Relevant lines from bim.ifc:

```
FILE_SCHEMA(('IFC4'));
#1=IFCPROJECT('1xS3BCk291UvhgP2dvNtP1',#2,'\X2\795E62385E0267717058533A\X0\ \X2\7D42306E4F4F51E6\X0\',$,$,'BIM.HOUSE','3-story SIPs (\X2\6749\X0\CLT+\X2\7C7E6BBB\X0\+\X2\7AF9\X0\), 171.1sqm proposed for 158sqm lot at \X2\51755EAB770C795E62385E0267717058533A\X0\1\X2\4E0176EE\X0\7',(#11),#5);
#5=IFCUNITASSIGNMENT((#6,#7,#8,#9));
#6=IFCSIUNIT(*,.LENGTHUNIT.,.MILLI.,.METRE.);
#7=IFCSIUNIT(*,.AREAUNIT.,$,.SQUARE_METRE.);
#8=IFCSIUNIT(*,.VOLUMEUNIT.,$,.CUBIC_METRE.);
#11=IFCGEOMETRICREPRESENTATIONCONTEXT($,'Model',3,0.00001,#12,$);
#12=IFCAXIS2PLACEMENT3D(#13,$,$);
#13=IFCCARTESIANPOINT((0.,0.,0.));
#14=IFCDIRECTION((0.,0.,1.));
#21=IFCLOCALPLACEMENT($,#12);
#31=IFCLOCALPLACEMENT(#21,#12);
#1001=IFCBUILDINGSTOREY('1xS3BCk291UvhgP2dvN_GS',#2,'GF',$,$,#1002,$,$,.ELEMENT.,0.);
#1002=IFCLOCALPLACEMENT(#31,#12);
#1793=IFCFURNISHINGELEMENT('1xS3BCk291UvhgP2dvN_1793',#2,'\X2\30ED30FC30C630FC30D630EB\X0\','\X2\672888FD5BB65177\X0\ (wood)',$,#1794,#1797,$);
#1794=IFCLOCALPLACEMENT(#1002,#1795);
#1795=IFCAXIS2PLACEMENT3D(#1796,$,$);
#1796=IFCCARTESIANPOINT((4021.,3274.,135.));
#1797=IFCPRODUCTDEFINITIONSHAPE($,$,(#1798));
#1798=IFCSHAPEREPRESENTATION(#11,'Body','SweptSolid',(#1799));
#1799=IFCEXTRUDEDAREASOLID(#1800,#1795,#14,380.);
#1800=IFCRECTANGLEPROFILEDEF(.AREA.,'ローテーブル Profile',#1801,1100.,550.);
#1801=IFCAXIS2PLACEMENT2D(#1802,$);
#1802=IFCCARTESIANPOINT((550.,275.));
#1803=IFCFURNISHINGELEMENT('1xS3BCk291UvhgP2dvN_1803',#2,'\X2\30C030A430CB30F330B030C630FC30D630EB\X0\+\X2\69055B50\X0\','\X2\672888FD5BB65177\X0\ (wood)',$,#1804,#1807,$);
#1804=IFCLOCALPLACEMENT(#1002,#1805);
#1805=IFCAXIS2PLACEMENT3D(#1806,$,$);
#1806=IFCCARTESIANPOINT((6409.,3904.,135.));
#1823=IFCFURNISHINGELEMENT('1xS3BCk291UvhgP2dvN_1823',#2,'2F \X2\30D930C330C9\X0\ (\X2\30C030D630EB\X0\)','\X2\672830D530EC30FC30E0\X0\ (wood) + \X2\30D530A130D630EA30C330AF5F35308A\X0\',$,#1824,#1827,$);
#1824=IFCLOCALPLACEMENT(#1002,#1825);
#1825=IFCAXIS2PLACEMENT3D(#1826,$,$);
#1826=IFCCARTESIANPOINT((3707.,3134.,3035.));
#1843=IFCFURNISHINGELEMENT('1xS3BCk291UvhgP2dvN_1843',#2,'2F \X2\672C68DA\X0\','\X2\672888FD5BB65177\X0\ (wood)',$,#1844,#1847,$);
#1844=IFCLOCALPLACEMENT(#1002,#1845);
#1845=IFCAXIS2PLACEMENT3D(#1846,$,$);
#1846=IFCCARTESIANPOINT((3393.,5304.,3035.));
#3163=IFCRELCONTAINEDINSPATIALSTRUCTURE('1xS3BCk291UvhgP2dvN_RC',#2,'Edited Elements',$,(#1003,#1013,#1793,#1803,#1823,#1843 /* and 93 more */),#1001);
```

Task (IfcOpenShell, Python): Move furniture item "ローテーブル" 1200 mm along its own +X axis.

```python
import ifcopenshell
import ifcopenshell.api.geometry
import ifcopenshell.util.placement
import ifcopenshell.util.unit

model = ifcopenshell.open("bim.ifc")
unit_scale = ifcopenshell.util.unit.calculate_unit_scale(model)

item = model.by_id(1793)
matrix = ifcopenshell.util.placement.get_local_placement(item.ObjectPlacement)
matrix[:3, 3] += matrix[:3, 0] * 1.2 / unit_scale
ifcopenshell.api.geometry.edit_object_placement(model, product=item, matrix=matrix, is_si=False)

print(ifcopenshell.util.placement.get_local_placement(item.ObjectPlacement).round(3) + 0.0)

model.write("bim_edited.ifc")
```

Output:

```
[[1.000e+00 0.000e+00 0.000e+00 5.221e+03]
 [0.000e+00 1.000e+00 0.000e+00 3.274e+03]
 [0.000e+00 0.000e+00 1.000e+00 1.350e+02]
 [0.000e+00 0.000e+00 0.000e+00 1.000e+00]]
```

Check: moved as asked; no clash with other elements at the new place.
